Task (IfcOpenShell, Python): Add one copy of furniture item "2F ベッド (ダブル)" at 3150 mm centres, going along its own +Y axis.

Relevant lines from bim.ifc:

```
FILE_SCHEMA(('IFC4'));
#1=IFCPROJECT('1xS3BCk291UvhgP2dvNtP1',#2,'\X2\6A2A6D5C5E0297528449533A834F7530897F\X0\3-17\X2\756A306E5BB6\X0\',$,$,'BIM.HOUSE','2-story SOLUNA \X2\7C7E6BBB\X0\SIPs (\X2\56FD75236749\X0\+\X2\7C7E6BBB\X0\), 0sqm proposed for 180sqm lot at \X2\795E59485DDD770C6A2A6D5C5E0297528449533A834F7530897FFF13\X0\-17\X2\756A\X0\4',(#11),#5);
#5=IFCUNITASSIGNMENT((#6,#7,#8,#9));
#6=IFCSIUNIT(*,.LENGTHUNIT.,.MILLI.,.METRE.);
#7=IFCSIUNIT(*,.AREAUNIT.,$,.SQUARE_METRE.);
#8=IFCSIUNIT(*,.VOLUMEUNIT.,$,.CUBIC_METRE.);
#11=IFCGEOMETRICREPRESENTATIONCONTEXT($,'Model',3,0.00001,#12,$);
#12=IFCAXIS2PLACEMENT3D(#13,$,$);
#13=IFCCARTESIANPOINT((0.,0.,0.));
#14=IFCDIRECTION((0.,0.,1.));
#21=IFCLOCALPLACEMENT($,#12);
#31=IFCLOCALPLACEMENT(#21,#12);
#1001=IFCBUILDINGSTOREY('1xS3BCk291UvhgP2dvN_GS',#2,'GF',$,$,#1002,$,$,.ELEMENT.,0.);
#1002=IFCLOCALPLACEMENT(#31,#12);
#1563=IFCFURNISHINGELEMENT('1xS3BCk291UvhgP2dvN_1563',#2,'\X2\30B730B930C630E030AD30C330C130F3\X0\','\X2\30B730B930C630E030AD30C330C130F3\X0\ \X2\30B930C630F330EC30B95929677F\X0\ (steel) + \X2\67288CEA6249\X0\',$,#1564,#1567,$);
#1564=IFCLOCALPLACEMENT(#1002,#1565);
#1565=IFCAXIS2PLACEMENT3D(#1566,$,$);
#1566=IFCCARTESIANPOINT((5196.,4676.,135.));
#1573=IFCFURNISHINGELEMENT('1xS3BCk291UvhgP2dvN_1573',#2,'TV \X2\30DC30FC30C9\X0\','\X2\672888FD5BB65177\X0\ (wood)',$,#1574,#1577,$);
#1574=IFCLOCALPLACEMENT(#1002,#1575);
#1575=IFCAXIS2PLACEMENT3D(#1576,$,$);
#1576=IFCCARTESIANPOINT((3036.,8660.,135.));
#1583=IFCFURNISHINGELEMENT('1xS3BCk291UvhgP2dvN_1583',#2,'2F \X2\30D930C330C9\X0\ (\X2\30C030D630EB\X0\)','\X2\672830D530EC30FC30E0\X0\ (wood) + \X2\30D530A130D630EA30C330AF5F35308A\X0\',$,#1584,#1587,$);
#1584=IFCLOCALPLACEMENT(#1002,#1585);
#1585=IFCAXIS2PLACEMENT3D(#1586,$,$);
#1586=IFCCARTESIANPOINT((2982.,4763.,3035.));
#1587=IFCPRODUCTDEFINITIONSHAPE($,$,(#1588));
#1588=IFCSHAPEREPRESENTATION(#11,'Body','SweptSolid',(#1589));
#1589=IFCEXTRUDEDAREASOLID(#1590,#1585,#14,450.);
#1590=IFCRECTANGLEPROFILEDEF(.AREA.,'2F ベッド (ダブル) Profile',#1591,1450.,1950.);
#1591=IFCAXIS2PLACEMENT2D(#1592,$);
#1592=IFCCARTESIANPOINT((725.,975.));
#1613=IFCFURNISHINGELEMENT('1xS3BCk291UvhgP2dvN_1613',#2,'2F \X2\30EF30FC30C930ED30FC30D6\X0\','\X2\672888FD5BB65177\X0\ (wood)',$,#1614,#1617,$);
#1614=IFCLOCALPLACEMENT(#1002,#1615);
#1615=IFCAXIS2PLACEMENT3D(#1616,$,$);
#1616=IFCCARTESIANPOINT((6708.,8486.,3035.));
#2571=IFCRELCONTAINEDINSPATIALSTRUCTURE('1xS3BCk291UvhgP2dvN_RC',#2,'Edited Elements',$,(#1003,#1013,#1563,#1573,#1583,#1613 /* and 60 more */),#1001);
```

```python
import ifcopenshell
import ifcopenshell.api.geometry
import ifcopenshell.api.root
import ifcopenshell.util.element
import ifcopenshell.util.placement
import ifcopenshell.util.unit

model = ifcopenshell.open("bim.ifc")
unit_scale = ifcopenshell.util.unit.calculate_unit_scale(model)


def reuse_history(source, copy):
    """copy_class also copies each property set's owner history, people and application; keep the originals."""
    for rel in copy.IsDefinedBy:
        if rel.is_a("IfcRelDefinesByProperties") and (history := rel.RelatingPropertyDefinition.OwnerHistory):
            rel.RelatingPropertyDefinition.OwnerHistory = source.OwnerHistory
            ifcopenshell.util.element.remove_deep2(model, history)


source = model.by_id(1583)
base = ifcopenshell.util.placement.get_local_placement(source.ObjectPlacement)
step = base[:3, 1] * 3.15 / unit_scale

for i in range(1, 2):
    copy = ifcopenshell.api.root.copy_class(model, product=source)
    copy.Representation = ifcopenshell.util.element.copy_deep(
        model, source.Representation, exclude=["IfcGeometricRepresentationContext", "IfcRepresentationMap"]
    )
    reuse_history(source, copy)
    matrix = base.copy()
    matrix[:3, 3] += i * step
    print("added at", matrix[:3, 3].round(3) + 0.0)
    ifcopenshell.api.geometry.edit_object_placement(model, product=copy, matrix=matrix, is_si=False)

model.write("bim_rev.ifc")
```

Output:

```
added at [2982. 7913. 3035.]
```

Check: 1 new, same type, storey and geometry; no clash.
